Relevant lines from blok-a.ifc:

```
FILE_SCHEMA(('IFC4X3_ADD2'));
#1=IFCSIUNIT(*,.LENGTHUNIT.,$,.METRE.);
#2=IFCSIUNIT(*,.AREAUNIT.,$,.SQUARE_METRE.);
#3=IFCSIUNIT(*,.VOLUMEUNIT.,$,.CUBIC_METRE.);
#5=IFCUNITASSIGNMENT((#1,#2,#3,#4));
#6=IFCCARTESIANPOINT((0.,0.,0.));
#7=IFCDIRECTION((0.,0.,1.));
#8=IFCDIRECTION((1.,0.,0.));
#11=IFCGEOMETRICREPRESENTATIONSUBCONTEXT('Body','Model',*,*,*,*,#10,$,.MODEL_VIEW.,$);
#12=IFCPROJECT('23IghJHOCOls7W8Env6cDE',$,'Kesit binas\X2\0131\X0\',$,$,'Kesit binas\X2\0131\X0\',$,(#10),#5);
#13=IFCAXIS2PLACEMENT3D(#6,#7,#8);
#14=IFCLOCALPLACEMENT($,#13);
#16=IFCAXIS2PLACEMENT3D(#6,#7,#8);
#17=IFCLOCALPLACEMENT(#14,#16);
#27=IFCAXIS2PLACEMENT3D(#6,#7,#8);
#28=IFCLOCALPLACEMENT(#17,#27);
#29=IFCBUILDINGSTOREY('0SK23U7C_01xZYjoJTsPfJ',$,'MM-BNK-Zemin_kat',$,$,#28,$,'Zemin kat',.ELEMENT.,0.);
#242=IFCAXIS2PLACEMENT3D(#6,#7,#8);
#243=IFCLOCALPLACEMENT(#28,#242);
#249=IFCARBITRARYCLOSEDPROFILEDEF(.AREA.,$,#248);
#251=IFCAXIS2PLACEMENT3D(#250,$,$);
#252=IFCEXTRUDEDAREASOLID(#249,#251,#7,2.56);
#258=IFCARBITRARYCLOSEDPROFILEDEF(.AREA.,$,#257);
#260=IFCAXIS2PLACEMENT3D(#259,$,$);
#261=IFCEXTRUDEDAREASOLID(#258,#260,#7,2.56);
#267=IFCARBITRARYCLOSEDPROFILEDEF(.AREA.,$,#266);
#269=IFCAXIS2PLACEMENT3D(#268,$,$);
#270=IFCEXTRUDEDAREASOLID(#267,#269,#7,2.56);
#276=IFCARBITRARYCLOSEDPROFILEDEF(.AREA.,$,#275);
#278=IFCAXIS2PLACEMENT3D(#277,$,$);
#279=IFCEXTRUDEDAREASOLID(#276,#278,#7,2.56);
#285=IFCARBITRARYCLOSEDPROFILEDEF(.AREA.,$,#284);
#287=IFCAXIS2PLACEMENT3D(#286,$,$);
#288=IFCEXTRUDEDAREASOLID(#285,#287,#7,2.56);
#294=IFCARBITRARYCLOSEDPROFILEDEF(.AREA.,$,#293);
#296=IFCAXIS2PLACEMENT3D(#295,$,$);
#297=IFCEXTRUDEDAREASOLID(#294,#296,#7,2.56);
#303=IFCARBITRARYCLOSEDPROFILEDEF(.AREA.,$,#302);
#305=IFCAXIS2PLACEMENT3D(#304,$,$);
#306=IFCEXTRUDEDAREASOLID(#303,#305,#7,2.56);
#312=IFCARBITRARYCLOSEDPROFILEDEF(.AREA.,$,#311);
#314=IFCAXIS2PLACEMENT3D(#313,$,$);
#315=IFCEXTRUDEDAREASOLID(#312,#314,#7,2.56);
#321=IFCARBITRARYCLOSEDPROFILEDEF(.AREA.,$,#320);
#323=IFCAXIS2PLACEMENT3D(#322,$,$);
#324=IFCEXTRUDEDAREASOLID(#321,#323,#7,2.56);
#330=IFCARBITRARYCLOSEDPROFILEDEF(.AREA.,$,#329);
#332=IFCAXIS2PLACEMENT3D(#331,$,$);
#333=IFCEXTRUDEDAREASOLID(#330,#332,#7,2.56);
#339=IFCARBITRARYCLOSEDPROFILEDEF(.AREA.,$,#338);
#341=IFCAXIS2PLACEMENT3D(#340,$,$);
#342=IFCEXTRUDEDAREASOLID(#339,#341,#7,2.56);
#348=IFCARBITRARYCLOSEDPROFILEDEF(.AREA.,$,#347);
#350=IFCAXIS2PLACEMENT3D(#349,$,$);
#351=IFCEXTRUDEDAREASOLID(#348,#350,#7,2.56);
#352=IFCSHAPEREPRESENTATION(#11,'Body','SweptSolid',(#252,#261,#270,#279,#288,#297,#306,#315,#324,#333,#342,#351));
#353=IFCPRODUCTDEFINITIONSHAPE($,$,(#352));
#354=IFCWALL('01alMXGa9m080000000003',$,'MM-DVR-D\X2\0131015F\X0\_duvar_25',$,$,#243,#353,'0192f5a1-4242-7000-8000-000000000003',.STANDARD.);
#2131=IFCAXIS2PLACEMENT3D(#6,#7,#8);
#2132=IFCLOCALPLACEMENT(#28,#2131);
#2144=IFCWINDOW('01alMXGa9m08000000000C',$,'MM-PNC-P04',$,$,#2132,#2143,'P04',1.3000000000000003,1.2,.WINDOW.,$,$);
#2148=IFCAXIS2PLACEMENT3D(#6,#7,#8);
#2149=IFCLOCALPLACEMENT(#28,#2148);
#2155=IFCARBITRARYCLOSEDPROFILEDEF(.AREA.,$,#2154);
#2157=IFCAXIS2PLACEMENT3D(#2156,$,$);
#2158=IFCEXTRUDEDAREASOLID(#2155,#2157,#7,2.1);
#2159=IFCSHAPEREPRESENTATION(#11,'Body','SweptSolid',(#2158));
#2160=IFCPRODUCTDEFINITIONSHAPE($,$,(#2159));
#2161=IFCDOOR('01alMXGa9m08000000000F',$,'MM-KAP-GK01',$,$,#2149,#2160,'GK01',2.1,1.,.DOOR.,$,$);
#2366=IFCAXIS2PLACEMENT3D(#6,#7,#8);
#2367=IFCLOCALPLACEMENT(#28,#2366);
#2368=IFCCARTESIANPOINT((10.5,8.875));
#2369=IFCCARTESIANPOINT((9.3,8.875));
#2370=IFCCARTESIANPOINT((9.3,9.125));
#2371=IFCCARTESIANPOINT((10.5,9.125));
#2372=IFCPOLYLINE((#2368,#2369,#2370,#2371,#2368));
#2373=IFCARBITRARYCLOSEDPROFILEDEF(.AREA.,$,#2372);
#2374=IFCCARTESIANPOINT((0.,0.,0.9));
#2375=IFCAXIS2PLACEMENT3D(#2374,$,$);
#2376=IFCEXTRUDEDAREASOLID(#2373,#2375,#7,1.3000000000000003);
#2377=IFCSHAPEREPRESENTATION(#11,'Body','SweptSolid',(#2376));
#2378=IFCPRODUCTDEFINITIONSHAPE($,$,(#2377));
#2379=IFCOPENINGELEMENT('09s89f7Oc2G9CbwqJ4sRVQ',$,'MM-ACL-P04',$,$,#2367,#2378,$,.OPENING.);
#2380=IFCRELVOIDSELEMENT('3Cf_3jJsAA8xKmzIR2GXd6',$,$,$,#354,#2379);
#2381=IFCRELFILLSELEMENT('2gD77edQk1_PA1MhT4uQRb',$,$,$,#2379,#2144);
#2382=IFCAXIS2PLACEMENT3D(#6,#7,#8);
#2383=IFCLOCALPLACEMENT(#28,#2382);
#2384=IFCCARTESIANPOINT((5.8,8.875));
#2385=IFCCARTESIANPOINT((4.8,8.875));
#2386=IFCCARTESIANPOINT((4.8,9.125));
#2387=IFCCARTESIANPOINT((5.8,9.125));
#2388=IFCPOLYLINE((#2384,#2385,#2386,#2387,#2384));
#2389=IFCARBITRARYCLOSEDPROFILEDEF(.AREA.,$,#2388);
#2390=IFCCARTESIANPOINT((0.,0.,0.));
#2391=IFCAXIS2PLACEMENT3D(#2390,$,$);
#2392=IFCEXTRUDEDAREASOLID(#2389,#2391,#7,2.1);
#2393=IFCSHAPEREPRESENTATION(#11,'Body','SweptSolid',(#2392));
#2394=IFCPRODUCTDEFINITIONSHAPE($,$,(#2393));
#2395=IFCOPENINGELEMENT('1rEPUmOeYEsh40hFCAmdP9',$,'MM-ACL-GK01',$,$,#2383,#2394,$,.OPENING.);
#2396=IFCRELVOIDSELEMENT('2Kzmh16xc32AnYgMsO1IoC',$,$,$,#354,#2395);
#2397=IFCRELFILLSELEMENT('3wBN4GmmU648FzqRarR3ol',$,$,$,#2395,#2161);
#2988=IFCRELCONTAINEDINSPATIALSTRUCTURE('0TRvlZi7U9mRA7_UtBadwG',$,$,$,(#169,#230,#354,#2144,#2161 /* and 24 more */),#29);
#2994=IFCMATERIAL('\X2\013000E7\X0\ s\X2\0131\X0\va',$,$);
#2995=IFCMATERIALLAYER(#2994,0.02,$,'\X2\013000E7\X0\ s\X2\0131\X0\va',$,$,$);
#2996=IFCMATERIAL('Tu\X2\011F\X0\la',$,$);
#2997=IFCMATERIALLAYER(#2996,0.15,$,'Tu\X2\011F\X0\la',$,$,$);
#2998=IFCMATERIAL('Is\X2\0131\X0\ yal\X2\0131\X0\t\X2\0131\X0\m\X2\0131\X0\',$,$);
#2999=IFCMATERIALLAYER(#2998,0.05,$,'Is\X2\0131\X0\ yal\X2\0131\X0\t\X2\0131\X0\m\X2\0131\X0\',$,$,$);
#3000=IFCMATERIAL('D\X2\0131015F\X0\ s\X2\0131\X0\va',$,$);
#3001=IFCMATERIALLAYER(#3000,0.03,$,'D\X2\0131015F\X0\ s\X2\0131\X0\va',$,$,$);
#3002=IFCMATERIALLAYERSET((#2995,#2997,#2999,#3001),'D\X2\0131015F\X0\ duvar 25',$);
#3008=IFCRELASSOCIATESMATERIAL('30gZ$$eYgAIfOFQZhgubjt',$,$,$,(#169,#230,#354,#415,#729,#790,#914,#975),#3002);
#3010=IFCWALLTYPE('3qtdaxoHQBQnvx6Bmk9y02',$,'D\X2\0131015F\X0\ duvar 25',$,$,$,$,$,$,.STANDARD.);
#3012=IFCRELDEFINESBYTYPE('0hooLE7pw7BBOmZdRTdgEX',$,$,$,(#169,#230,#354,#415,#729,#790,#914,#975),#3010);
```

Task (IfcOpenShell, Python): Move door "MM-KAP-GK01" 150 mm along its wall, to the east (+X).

```python
import ifcopenshell
import ifcopenshell.api.geometry
import ifcopenshell.util.placement

model = ifcopenshell.open("blok-a.ifc")

door = model.by_id(2161)
opening = door.FillsVoids[0].RelatingOpeningElement
wall = opening.VoidsElements[0].RelatingBuildingElement

wall_matrix = ifcopenshell.util.placement.get_local_placement(wall.ObjectPlacement)
shift = wall_matrix[:3, 0] * 0.15
before = ifcopenshell.util.placement.get_local_placement(door.ObjectPlacement)[:3, 3].copy()

# The door is not placed relative to its opening, so move both.
for product in (opening, door):
    matrix = ifcopenshell.util.placement.get_local_placement(product.ObjectPlacement)
    matrix[:3, 3] += shift
    ifcopenshell.api.geometry.edit_object_placement(model, product=product, matrix=matrix, is_si=False)

after = ifcopenshell.util.placement.get_local_placement(door.ObjectPlacement)[:3, 3]
print("door moved by", (after - before).round(3) + 0.0)

model.write("blok-a_v2.ifc")
```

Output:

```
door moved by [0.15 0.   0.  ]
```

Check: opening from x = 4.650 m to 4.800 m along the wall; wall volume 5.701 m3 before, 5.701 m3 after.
